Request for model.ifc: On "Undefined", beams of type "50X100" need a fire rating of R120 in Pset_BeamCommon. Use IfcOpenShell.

First a look at what the model holds.

```python
import ifcopenshell
import ifcopenshell.util.element

model = ifcopenshell.open("model.ifc")
print(model.schema)
storey = next(s for s in model.by_type("IfcBuildingStorey") if s.Name == "Undefined")
beams = [e for e in ifcopenshell.util.element.get_decomposition(storey) if e.is_a("IfcBeam")]
seen = {}
for e in beams:
    element_type = ifcopenshell.util.element.get_type(e)
    key = (element_type.Name if element_type != e and element_type else None, ifcopenshell.util.element.get_pset(e, "Pset_BeamCommon", "FireRating"))
    seen[key] = seen.get(key, 0) + 1
for (name, value), count in sorted(seen.items(), key=str):
    print(count, "x", name, "|", value)
```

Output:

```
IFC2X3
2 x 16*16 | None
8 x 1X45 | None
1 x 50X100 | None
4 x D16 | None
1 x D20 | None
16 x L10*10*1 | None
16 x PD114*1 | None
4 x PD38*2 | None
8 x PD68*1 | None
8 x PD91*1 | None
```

```python
import ifcopenshell
import ifcopenshell.api.pset
import ifcopenshell.util.element

model = ifcopenshell.open("model.ifc")

storey = next(s for s in model.by_type("IfcBuildingStorey") if s.Name == "Undefined")
beams = [e for e in ifcopenshell.util.element.get_decomposition(storey) if e.is_a("IfcBeam")]

count = 0
for e in beams:
    element_type = ifcopenshell.util.element.get_type(e)
    if element_type in (None, e) or element_type.Name != "50X100":
        continue
    # add_pset returns the element's existing set when there is one.
    pset = ifcopenshell.api.pset.add_pset(model, product=e, name="Pset_BeamCommon")
    ifcopenshell.api.pset.edit_pset(model, pset=pset, properties={"FireRating": "R120"})
    count += 1

print(count, "beams updated")

model.write("model_edited.ifc")
```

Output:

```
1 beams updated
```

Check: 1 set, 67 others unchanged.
